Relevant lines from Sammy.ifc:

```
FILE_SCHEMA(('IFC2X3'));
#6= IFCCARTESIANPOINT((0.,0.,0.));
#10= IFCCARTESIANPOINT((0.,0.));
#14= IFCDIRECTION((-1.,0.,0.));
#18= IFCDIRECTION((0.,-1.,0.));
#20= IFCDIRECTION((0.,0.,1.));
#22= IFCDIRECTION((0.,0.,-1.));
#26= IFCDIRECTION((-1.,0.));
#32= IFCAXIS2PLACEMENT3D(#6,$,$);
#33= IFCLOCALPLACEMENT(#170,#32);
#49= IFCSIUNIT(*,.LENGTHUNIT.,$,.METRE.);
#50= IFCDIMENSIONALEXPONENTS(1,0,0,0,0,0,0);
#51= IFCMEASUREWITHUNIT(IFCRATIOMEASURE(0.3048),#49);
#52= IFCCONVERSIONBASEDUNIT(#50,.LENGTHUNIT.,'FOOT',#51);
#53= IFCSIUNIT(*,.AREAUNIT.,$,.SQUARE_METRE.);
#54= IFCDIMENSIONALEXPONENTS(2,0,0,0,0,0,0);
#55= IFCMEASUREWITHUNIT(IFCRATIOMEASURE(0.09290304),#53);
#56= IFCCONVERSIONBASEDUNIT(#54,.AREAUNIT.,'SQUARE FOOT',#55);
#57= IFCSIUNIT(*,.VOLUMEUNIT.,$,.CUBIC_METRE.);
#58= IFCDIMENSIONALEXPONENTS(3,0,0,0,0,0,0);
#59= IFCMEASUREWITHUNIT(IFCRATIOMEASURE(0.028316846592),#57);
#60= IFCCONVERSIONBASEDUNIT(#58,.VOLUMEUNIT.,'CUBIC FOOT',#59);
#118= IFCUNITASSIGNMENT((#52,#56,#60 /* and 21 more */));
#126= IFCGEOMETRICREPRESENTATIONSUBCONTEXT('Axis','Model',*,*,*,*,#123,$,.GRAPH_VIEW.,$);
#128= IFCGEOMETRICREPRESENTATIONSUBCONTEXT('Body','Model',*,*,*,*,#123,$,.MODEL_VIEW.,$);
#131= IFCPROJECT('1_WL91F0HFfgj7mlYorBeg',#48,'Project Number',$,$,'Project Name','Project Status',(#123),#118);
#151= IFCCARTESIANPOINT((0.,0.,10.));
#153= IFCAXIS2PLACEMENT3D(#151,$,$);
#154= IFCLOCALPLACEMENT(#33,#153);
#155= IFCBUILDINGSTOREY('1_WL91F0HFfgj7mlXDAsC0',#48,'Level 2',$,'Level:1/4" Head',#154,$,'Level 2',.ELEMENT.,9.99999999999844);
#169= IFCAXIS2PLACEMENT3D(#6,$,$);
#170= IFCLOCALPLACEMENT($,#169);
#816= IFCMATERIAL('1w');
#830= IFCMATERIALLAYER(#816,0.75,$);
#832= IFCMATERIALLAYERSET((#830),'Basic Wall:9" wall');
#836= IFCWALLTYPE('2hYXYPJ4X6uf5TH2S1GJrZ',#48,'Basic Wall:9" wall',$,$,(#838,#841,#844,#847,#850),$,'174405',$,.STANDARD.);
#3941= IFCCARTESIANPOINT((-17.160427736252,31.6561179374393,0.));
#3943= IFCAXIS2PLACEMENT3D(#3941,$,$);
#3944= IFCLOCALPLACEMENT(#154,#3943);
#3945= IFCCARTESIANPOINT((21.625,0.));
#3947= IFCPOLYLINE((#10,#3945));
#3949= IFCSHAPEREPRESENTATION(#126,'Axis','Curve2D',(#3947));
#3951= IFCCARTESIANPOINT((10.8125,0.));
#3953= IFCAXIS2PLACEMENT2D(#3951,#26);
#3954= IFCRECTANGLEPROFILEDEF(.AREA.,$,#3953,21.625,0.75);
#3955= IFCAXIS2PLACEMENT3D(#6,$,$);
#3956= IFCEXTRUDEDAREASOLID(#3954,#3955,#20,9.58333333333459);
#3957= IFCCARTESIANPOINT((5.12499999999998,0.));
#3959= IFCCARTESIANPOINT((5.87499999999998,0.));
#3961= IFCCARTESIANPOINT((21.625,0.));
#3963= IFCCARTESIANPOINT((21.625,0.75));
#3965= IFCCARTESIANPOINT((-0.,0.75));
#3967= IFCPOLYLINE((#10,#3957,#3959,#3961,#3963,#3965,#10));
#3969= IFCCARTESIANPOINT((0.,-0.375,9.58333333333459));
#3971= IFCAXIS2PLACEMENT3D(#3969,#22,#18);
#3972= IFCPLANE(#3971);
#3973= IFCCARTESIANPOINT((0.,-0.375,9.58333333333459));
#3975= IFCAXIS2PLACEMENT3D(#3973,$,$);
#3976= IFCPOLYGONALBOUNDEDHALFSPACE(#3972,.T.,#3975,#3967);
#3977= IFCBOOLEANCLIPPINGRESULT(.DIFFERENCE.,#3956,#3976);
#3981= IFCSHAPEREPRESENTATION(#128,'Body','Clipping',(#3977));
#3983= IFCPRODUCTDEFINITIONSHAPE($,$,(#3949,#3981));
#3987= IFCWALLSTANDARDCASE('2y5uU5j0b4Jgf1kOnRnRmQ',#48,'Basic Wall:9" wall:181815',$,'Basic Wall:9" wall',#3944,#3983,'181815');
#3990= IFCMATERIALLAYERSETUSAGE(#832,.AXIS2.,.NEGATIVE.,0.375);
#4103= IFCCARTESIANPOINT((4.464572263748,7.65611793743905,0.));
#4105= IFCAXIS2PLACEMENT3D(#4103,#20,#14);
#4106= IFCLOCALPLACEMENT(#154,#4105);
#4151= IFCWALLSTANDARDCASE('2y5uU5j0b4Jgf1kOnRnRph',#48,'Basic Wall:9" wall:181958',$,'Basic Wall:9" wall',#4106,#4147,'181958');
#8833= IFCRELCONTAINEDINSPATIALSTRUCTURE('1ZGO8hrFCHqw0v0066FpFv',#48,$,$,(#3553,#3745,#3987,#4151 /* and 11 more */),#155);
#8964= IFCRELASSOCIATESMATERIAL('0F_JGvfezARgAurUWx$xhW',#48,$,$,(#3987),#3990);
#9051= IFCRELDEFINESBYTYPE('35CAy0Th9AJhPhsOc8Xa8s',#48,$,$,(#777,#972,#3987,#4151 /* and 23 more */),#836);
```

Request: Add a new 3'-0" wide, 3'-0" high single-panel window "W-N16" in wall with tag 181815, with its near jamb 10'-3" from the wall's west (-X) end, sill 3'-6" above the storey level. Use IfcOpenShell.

```python
import numpy as np
import ifcopenshell
import ifcopenshell.api.feature
import ifcopenshell.api.geometry
import ifcopenshell.api.root
import ifcopenshell.api.spatial
import ifcopenshell.api.type
import ifcopenshell.geom
import ifcopenshell.util.element
import ifcopenshell.util.placement
import ifcopenshell.util.representation
import ifcopenshell.util.shape
import ifcopenshell.util.unit

model = ifcopenshell.open("Sammy.ifc")
unit_scale = ifcopenshell.util.unit.calculate_unit_scale(model)
settings = ifcopenshell.geom.settings()


def volume(element):
    """Net volume in cubic metres, openings subtracted."""
    shape = ifcopenshell.geom.create_shape(settings, element)
    return ifcopenshell.util.shape.get_volume(shape.geometry)


wall = model.by_guid("2y5uU5j0b4Jgf1kOnRnRmQ")
storey = ifcopenshell.util.element.get_container(wall, ifc_class="IfcBuildingStorey")
context = ifcopenshell.util.representation.get_context(model, "Model", "Body", "MODEL_VIEW")
before = volume(wall)

width, height, from_end, sill = 0.9144, 0.9144, 3.1242, 1.0668  # metres

# The wall runs along its own X axis, and the end named is its -X end.
wall_shape = ifcopenshell.geom.create_shape(settings, wall)
x, y, z = ifcopenshell.util.shape.get_vertices(wall_shape.geometry).T
start = x.min() + from_end
face, thickness = float(y.min()), float(y.max() - y.min())
wall_matrix = ifcopenshell.util.placement.get_local_placement(wall.ObjectPlacement)
level = ifcopenshell.util.placement.get_local_placement(storey.ObjectPlacement)[2, 3]


def in_wall(x, y):
    """Placement at x, y metres in the wall's axes, at sill height."""
    matrix = wall_matrix.copy()
    matrix[:, 3] = wall_matrix @ np.array([x / unit_scale, y / unit_scale, 0.0, 1.0])
    matrix[2, 3] = level + sill / unit_scale
    return matrix


# Opening: a box that overshoots both wall faces by 50 mm.
opening = ifcopenshell.api.root.create_entity(model, ifc_class="IfcOpeningElement")
box = ifcopenshell.api.geometry.add_wall_representation(
    model, context=context, length=width, height=height, thickness=thickness + 0.1
)
ifcopenshell.api.geometry.assign_representation(model, product=opening, representation=box)
ifcopenshell.api.geometry.edit_object_placement(model, product=opening, matrix=in_wall(start, face - 0.05), is_si=False)
ifcopenshell.api.feature.add_feature(model, feature=opening, element=wall)

window = ifcopenshell.api.root.create_entity(model, ifc_class="IfcWindow", name="W-N16")
window.OverallWidth, window.OverallHeight = width / unit_scale, height / unit_scale
body = ifcopenshell.api.geometry.add_window_representation(
    model,
    context=context,
    overall_width=window.OverallWidth,
    overall_height=window.OverallHeight,
    partition_type="SINGLE_PANEL",
)
ifcopenshell.api.geometry.assign_representation(model, product=window, representation=body)
ifcopenshell.api.spatial.assign_container(model, products=[window], relating_structure=storey)
fills = ifcopenshell.api.feature.add_filling(model, opening=opening, element=window)
fills.OwnerHistory = window.OwnerHistory  # required in IFC2X3

# IFC2X3 keeps the operation on the window style.
style = ifcopenshell.api.root.create_entity(model, ifc_class="IfcWindowStyle", name="W-N16")
style.OperationType, style.ConstructionType = "SINGLE_PANEL", "NOTDEFINED"
style.ParameterTakesPrecedence = style.Sizeable = False
ifcopenshell.api.type.assign_type(model, related_objects=[window], relating_type=style)

# Centre the window in the wall's thickness.
ifcopenshell.api.geometry.edit_object_placement(model, product=window, matrix=in_wall(start, face), is_si=False)
window_shape = ifcopenshell.geom.create_shape(settings, window)
depth = ifcopenshell.util.shape.get_vertices(window_shape.geometry)[:, 1]
offset = face + thickness / 2 - (depth.min() + depth.max()) / 2
ifcopenshell.api.geometry.edit_object_placement(model, product=window, matrix=in_wall(start, offset), is_si=False)

after = volume(wall)

print(f"wall volume {before:.3f} -> {after:.3f} m3")

model.write("Sammy_v2.ifc")
```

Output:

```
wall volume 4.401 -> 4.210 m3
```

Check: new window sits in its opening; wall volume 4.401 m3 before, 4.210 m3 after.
